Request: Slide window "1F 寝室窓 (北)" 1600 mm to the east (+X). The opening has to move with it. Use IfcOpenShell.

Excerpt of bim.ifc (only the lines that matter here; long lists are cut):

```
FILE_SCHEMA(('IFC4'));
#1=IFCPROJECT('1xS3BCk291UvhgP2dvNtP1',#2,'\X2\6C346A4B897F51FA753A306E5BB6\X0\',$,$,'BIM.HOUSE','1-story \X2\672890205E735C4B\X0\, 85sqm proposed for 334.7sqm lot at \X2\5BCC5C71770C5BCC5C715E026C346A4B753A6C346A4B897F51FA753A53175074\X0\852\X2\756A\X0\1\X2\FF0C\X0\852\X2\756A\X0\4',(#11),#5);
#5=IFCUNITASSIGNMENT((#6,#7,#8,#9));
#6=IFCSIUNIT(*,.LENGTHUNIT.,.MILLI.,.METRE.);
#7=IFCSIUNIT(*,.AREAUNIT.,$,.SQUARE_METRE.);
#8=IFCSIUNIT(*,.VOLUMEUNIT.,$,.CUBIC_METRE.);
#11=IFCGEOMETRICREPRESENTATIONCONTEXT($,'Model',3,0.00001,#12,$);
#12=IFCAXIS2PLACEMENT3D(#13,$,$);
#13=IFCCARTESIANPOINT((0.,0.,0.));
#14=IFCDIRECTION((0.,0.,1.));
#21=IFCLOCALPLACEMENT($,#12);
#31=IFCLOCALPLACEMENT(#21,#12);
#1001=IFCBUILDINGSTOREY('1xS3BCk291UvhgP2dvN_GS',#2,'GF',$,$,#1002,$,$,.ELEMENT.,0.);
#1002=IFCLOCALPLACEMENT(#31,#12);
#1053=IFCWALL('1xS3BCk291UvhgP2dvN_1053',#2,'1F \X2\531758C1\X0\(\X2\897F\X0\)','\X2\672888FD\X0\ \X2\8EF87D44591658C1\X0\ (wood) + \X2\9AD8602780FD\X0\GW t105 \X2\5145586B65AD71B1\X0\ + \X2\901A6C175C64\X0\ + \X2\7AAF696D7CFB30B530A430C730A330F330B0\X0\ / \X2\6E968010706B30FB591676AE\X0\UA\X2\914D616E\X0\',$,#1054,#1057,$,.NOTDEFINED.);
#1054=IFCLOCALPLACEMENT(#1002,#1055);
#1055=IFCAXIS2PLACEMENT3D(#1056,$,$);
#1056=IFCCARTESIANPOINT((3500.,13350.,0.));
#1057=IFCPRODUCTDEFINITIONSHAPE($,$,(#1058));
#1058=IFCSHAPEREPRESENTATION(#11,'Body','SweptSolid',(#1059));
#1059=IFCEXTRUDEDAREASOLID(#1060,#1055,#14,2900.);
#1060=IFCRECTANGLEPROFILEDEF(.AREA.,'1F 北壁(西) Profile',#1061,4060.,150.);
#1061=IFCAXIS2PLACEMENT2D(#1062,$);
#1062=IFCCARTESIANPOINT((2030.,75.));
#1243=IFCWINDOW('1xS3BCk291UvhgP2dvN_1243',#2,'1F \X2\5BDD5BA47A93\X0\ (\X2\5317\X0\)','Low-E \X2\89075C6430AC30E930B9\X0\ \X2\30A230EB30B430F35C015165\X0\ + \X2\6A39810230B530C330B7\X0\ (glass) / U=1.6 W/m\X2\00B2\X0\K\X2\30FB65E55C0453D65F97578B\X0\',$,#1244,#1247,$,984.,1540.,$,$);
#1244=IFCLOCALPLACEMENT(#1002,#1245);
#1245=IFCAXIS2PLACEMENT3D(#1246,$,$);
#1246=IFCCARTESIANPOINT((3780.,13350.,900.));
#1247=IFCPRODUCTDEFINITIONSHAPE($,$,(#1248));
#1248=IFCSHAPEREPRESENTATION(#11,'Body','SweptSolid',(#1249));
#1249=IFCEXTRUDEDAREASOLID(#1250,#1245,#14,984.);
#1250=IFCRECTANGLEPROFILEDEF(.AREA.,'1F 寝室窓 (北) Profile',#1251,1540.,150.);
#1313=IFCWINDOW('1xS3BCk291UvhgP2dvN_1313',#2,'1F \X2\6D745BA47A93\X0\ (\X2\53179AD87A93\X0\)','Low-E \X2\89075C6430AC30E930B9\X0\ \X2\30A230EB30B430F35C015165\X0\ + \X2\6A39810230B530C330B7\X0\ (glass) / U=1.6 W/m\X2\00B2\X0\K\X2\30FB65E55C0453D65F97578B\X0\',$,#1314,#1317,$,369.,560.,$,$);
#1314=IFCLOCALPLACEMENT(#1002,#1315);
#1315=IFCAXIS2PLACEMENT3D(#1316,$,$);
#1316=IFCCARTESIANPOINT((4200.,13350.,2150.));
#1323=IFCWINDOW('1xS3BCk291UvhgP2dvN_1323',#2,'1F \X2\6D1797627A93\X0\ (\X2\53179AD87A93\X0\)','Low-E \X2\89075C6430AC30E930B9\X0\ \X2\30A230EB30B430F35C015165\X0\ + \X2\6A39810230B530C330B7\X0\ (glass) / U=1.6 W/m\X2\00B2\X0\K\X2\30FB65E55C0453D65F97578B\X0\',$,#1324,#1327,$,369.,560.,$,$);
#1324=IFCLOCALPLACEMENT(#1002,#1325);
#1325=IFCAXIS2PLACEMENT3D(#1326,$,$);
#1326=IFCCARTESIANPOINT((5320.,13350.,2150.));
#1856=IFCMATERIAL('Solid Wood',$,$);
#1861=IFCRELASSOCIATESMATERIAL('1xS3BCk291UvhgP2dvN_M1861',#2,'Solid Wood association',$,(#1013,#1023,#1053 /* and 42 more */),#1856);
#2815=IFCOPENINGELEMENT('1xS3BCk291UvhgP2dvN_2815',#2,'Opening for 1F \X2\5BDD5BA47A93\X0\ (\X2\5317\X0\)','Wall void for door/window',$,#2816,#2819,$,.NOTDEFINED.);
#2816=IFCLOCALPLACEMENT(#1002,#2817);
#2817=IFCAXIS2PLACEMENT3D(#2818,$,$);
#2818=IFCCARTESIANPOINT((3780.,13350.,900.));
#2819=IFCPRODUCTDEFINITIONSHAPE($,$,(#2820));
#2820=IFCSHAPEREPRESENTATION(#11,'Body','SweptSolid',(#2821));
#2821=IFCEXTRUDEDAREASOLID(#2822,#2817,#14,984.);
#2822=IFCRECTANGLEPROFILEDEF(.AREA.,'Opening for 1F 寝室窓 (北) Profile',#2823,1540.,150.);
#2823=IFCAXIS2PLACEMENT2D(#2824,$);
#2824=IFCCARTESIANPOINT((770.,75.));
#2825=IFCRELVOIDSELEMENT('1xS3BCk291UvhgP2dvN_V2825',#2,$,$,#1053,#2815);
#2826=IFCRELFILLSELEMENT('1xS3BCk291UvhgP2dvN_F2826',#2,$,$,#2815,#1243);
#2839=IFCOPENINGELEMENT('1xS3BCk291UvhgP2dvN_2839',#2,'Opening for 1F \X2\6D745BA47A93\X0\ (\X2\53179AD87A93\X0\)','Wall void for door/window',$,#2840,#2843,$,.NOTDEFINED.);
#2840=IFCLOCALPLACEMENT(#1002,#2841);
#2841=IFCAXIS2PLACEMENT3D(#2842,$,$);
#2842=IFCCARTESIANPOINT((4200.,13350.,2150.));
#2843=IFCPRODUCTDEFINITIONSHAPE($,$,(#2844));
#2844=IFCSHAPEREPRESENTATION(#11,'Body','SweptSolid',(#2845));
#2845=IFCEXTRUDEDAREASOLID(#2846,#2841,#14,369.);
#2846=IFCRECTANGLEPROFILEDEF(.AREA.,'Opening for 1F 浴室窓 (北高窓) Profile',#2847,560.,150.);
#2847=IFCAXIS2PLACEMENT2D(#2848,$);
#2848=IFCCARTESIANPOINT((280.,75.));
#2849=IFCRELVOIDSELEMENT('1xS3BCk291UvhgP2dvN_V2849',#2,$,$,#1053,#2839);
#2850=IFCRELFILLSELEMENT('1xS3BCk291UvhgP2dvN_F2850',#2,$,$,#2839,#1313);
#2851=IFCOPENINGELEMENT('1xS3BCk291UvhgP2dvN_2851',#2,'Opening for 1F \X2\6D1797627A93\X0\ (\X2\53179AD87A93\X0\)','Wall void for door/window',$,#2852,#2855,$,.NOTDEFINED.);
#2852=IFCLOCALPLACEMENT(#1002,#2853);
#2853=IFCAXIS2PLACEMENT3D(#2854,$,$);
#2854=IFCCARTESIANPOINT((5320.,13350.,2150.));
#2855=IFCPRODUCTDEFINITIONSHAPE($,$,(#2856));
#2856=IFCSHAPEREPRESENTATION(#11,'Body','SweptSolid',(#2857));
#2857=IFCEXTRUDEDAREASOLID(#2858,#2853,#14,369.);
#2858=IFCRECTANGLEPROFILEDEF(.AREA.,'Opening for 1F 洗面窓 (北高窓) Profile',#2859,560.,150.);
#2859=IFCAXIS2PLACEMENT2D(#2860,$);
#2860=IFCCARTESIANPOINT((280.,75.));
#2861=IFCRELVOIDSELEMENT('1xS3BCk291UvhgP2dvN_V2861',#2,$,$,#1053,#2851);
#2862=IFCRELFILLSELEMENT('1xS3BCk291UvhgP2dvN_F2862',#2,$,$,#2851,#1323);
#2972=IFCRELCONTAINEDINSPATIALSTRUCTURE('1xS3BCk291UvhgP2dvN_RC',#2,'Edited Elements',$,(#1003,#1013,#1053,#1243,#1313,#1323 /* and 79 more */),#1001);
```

```python
import ifcopenshell
import ifcopenshell.api.geometry
import ifcopenshell.util.placement
import ifcopenshell.util.unit

model = ifcopenshell.open("bim.ifc")
unit_scale = ifcopenshell.util.unit.calculate_unit_scale(model)

window = model.by_id(1243)
opening = window.FillsVoids[0].RelatingOpeningElement
wall = opening.VoidsElements[0].RelatingBuildingElement

wall_matrix = ifcopenshell.util.placement.get_local_placement(wall.ObjectPlacement)
shift = wall_matrix[:3, 0] * 1.6 / unit_scale
before = ifcopenshell.util.placement.get_local_placement(window.ObjectPlacement)[:3, 3].copy()

# The window is not placed relative to its opening, so move both.
for product in (opening, window):
    matrix = ifcopenshell.util.placement.get_local_placement(product.ObjectPlacement)
    matrix[:3, 3] += shift
    ifcopenshell.api.geometry.edit_object_placement(model, product=product, matrix=matrix, is_si=False)

after = ifcopenshell.util.placement.get_local_placement(window.ObjectPlacement)[:3, 3]
print("window moved by", (after - before).round(3) + 0.0)

model.write("bim_edited.ifc")
```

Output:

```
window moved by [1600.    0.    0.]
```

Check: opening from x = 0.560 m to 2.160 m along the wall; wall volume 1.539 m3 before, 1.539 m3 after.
